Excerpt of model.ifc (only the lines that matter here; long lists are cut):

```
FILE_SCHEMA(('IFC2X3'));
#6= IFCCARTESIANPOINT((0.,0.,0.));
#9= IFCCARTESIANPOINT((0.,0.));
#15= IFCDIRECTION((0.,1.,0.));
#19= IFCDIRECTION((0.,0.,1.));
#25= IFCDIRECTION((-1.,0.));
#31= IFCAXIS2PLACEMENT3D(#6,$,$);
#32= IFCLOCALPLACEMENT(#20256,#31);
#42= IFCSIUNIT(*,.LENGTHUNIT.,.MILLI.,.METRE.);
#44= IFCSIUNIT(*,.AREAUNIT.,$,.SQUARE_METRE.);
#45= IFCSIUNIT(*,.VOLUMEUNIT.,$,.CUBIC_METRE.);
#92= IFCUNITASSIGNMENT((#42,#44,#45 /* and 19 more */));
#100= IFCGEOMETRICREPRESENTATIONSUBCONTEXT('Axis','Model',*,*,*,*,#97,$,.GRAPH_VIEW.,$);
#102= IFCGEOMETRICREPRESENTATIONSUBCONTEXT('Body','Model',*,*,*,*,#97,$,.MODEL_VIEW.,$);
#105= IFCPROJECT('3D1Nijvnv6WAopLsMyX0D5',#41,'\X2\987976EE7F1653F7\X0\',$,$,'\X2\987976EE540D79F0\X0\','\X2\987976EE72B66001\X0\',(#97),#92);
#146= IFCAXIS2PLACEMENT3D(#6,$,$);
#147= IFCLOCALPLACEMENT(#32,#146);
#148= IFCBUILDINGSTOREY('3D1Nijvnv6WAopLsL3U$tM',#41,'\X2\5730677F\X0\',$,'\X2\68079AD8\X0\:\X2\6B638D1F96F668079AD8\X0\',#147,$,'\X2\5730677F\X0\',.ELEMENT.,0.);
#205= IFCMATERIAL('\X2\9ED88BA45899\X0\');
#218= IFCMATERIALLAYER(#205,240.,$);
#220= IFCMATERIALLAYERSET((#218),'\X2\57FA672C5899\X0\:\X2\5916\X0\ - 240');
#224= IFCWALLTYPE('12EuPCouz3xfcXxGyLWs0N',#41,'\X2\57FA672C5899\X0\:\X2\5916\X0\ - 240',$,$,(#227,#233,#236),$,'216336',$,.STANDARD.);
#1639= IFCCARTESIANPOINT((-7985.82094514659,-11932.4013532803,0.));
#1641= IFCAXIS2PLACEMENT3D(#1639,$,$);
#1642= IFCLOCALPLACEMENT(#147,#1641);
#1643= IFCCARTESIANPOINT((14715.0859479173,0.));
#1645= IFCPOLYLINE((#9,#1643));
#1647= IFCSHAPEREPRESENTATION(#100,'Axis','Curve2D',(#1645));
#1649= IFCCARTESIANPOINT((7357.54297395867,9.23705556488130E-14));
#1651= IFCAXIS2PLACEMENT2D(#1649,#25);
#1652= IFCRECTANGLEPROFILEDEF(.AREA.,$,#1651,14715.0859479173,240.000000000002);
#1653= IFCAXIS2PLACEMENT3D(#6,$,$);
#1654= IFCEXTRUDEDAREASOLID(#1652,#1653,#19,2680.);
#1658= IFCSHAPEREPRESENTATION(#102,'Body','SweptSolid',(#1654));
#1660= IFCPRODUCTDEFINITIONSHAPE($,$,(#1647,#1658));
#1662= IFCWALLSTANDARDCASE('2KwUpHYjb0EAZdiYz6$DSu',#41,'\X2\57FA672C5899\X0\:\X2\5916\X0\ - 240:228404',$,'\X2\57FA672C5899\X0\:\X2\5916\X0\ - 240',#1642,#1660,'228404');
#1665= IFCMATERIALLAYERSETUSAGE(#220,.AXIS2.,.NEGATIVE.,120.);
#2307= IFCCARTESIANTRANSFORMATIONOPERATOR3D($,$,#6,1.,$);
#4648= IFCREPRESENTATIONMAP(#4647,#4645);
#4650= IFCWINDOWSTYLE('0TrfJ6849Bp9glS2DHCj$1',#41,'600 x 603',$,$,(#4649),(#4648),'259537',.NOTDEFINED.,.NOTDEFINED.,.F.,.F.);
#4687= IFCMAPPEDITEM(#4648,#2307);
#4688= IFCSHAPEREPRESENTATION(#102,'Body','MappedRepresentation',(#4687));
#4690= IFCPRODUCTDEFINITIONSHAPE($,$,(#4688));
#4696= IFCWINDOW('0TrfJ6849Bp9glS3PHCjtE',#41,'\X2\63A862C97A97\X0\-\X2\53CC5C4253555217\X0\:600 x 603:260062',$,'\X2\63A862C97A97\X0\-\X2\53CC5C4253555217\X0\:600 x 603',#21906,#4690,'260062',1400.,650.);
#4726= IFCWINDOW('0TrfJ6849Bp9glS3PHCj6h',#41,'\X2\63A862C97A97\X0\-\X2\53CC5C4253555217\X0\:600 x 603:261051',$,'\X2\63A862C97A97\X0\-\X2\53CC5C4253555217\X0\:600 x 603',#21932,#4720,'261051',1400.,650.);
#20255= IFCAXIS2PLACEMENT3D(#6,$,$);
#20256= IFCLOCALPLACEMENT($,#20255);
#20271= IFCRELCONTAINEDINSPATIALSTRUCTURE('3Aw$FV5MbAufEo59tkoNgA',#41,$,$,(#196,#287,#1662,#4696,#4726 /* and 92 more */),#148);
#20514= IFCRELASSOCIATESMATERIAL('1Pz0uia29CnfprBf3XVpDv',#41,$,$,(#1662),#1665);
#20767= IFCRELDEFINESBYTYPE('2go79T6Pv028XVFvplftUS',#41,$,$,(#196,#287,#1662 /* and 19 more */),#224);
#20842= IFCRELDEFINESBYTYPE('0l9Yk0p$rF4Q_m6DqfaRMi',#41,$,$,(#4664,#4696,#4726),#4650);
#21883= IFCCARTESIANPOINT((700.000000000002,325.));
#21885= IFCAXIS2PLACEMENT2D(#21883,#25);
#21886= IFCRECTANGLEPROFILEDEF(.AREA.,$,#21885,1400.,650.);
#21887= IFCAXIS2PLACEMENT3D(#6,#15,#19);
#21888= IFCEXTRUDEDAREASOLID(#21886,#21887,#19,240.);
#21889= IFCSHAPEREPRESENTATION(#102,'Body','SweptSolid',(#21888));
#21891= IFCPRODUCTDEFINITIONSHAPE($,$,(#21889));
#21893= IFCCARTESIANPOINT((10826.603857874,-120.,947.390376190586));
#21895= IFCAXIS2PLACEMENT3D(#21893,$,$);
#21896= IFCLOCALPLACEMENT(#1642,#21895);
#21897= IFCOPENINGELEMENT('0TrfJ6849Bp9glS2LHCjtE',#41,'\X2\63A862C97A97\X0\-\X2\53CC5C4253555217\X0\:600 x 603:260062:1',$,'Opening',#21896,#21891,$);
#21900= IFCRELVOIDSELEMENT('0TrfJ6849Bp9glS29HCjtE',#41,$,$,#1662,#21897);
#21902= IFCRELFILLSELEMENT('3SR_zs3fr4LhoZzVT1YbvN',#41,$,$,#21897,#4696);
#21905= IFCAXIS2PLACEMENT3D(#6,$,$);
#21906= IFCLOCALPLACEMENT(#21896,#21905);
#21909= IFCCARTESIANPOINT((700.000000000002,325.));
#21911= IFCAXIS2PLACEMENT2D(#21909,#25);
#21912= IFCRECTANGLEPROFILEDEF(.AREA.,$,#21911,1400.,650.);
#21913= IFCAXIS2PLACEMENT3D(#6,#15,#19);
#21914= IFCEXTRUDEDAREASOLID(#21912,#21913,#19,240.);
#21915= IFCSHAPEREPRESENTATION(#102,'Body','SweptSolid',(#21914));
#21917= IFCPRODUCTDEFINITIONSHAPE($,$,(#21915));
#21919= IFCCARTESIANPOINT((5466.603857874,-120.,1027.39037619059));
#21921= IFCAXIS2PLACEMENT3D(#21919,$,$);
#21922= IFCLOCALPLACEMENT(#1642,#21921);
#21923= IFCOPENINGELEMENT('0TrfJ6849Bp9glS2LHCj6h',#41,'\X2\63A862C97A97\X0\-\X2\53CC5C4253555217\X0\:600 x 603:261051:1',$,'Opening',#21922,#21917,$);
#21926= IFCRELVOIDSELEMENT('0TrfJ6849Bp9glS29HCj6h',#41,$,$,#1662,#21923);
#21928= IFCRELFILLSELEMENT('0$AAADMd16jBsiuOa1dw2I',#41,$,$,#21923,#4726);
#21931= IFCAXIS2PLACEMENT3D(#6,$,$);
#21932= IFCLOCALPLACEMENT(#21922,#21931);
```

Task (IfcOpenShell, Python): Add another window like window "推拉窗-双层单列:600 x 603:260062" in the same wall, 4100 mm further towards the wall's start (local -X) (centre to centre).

```python
import ifcopenshell
import ifcopenshell.api.feature
import ifcopenshell.api.geometry
import ifcopenshell.api.root
import ifcopenshell.geom
import ifcopenshell.util.element
import ifcopenshell.util.placement
import ifcopenshell.util.shape

model = ifcopenshell.open("model.ifc")
settings = ifcopenshell.geom.settings()


def volume(element):
    """Net volume in cubic metres, openings subtracted."""
    shape = ifcopenshell.geom.create_shape(settings, element)
    return ifcopenshell.util.shape.get_volume(shape.geometry)


def reuse_history(source, copy):
    """copy_class also copies each property set's owner history, people and application; keep the originals."""
    for rel in copy.IsDefinedBy:
        if rel.is_a("IfcRelDefinesByProperties") and (history := rel.RelatingPropertyDefinition.OwnerHistory):
            rel.RelatingPropertyDefinition.OwnerHistory = source.OwnerHistory
            ifcopenshell.util.element.remove_deep2(model, history)


window = model.by_guid("0TrfJ6849Bp9glS3PHCjtE")
opening = window.FillsVoids[0].RelatingOpeningElement
wall = opening.VoidsElements[0].RelatingBuildingElement
before = volume(wall)
shift = ifcopenshell.util.placement.get_local_placement(wall.ObjectPlacement)[:3, 0] * -4100.0

# copy_class copies the void relationship, type, container and properties, but no geometry.
new_opening = ifcopenshell.api.root.copy_class(model, product=opening)
new_opening.Representation = ifcopenshell.util.element.copy_deep(
    model, opening.Representation, exclude=["IfcGeometricRepresentationContext", "IfcRepresentationMap"]
)
new_opening.Name = "推拉窗-双层单列:600 x 603"
new_window = ifcopenshell.api.root.copy_class(model, product=window)
new_window.Representation = ifcopenshell.util.element.copy_deep(
    model, window.Representation, exclude=["IfcGeometricRepresentationContext", "IfcRepresentationMap"]
)
new_window.Name = "推拉窗-双层单列:600 x 603"
new_window.Tag = None
reuse_history(window, new_window)
fills = ifcopenshell.api.feature.add_filling(model, opening=new_opening, element=new_window)
fills.OwnerHistory = new_window.OwnerHistory  # required in IFC2X3

for old, new in ((opening, new_opening), (window, new_window)):
    matrix = ifcopenshell.util.placement.get_local_placement(old.ObjectPlacement)
    matrix[:3, 3] += shift
    ifcopenshell.api.geometry.edit_object_placement(model, product=new, matrix=matrix, is_si=False)

after = volume(wall)

print(f"wall volume {before:.3f} -> {after:.3f} m3")

model.write("model_updated.ifc")
```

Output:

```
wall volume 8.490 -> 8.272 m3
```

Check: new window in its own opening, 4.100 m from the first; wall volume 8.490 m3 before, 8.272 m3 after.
